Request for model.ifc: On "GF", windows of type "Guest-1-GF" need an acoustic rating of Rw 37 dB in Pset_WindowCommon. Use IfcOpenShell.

First a look at what the model holds.

```python
import ifcopenshell
import ifcopenshell.util.element

model = ifcopenshell.open("model.ifc")
print(model.schema)
storey = next(s for s in model.by_type("IfcBuildingStorey") if s.Name == "GF")
windows = [e for e in ifcopenshell.util.element.get_decomposition(storey) if e.is_a("IfcWindow")]
seen = {}
for e in windows:
    element_type = ifcopenshell.util.element.get_type(e)
    key = (element_type.Name if element_type != e and element_type else None, ifcopenshell.util.element.get_pset(e, "Pset_WindowCommon", "AcousticRating"))
    seen[key] = seen.get(key, 0) + 1
for (name, value), count in sorted(seen.items(), key=str):
    print(count, "x", name, "|", value)
```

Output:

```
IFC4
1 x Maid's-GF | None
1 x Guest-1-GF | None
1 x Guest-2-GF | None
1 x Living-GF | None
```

```python
import ifcopenshell
import ifcopenshell.api.pset
import ifcopenshell.util.element

model = ifcopenshell.open("model.ifc")

storey = next(s for s in model.by_type("IfcBuildingStorey") if s.Name == "GF")
windows = [e for e in ifcopenshell.util.element.get_decomposition(storey) if e.is_a("IfcWindow")]

count = 0
for e in windows:
    element_type = ifcopenshell.util.element.get_type(e)
    if element_type in (None, e) or element_type.Name != "Guest-1-GF":
        continue
    # add_pset returns the element's existing set when there is one.
    pset = ifcopenshell.api.pset.add_pset(model, product=e, name="Pset_WindowCommon")
    ifcopenshell.api.pset.edit_pset(model, pset=pset, properties={"AcousticRating": "Rw 37 dB"})
    count += 1

print(count, "windows updated")

model.write("model_rev.ifc")
```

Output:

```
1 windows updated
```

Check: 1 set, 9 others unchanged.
